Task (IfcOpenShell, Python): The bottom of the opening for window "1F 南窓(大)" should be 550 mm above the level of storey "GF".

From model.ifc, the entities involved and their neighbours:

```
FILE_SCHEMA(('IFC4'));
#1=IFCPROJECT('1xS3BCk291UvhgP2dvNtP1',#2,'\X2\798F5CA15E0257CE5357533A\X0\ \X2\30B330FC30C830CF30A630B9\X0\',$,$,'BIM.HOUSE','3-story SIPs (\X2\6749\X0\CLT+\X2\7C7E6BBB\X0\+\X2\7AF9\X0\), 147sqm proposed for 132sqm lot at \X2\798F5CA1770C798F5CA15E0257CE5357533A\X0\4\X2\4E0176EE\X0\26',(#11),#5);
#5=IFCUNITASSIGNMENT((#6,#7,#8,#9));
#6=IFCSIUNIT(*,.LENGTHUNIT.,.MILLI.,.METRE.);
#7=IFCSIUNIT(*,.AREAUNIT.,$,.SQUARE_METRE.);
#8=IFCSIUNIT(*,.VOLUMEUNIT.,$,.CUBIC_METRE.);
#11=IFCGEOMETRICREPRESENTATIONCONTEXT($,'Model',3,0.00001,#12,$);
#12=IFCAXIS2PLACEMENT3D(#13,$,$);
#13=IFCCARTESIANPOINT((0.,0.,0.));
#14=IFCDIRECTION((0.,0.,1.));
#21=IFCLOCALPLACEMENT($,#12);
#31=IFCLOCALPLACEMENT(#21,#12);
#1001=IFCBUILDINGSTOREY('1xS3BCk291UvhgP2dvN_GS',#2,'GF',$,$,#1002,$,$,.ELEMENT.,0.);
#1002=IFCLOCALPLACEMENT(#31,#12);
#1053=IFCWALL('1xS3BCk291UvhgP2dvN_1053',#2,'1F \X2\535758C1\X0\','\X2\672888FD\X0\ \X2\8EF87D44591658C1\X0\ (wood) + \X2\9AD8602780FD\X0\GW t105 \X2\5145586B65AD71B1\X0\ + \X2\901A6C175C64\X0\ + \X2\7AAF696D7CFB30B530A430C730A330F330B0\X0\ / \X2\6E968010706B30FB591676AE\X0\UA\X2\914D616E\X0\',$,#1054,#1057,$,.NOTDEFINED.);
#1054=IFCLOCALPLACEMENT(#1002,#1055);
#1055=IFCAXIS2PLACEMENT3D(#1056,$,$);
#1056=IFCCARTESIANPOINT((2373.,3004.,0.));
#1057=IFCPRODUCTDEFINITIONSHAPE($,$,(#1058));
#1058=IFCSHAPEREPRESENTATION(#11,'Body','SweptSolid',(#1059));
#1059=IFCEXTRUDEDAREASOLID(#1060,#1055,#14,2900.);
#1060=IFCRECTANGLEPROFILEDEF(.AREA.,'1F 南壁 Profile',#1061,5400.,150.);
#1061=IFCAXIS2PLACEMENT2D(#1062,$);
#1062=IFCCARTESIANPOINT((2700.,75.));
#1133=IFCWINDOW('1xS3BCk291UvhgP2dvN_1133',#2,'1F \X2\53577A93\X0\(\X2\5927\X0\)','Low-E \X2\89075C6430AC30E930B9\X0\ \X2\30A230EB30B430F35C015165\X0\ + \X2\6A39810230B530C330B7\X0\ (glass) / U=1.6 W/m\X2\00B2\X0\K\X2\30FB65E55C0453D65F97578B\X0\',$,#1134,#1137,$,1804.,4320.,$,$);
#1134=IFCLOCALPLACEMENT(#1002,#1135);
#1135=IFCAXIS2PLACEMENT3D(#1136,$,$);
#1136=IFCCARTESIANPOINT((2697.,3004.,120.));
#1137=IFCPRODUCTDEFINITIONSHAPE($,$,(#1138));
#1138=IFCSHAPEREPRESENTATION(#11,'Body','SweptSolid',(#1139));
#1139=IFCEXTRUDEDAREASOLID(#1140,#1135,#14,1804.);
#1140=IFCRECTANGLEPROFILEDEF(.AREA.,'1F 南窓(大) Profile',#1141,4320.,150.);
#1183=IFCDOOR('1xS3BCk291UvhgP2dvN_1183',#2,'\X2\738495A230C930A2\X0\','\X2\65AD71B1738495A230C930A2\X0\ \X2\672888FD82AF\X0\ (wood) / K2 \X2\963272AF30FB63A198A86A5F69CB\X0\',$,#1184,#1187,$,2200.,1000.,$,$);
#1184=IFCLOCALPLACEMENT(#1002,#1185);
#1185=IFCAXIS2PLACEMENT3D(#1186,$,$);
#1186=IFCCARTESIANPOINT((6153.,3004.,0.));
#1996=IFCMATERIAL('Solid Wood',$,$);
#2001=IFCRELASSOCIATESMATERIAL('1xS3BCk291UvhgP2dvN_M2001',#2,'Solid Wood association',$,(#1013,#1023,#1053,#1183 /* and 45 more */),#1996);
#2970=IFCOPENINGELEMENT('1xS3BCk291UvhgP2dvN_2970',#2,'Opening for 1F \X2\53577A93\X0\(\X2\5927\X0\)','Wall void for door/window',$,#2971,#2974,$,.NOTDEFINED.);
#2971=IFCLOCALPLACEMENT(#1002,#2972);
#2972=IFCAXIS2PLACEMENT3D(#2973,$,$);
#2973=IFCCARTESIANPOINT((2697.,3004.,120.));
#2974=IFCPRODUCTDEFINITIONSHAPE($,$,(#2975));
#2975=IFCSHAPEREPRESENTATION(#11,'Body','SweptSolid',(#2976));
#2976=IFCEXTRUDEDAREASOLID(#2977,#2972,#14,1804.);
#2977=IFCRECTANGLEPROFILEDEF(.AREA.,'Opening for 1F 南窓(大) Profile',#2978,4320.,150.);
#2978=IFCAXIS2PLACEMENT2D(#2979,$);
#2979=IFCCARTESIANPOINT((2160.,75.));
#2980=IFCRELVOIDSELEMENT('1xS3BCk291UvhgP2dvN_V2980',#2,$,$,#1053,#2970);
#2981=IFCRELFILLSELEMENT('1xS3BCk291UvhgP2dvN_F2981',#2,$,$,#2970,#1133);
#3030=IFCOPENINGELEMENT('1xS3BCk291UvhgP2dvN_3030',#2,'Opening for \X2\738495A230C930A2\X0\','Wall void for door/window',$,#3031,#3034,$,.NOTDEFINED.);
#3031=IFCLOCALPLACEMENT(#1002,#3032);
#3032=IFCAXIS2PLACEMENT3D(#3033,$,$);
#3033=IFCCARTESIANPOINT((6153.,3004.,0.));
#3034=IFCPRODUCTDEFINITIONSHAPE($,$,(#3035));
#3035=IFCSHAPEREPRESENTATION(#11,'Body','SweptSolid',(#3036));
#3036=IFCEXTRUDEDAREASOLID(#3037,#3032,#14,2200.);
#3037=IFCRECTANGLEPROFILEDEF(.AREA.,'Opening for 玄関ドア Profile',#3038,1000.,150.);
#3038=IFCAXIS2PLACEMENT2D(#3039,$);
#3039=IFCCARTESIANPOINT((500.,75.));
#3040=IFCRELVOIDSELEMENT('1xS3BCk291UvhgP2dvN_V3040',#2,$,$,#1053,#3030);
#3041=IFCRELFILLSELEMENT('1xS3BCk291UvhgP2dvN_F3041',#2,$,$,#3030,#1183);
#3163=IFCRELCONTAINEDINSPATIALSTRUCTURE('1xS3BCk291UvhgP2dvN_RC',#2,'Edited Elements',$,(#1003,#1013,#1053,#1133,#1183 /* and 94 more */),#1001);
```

```python
import numpy as np
import ifcopenshell
import ifcopenshell.api.geometry
import ifcopenshell.geom
import ifcopenshell.util.element
import ifcopenshell.util.placement
import ifcopenshell.util.shape
import ifcopenshell.util.unit

model = ifcopenshell.open("model.ifc")
unit_scale = ifcopenshell.util.unit.calculate_unit_scale(model)

window = model.by_guid("1xS3BCk291UvhgP2dvN_1133")
opening = window.FillsVoids[0].RelatingOpeningElement
storey = ifcopenshell.util.element.get_container(window, ifc_class="IfcBuildingStorey")
level = ifcopenshell.util.placement.get_local_placement(storey.ObjectPlacement)[2, 3]

# The opening's origin need not be at the sill, so measure its lowest point.
shape = ifcopenshell.geom.create_shape(ifcopenshell.geom.settings(), opening)
bottom = ifcopenshell.util.shape.get_shape_bottom_elevation(shape, shape.geometry) / unit_scale
dz = level + 0.55 / unit_scale - bottom

shift = np.array([0.0, 0.0, dz])
# The window is not placed relative to its opening, so move both.
for product in (opening, window):
    matrix = ifcopenshell.util.placement.get_local_placement(product.ObjectPlacement)
    matrix[:3, 3] += shift
    ifcopenshell.api.geometry.edit_object_placement(model, product=product, matrix=matrix, is_si=False)

print(f"moved by {dz * unit_scale:+.3f} m")

model.write("model_edited.ifc")
```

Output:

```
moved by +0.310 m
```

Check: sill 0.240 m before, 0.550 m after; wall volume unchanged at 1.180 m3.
